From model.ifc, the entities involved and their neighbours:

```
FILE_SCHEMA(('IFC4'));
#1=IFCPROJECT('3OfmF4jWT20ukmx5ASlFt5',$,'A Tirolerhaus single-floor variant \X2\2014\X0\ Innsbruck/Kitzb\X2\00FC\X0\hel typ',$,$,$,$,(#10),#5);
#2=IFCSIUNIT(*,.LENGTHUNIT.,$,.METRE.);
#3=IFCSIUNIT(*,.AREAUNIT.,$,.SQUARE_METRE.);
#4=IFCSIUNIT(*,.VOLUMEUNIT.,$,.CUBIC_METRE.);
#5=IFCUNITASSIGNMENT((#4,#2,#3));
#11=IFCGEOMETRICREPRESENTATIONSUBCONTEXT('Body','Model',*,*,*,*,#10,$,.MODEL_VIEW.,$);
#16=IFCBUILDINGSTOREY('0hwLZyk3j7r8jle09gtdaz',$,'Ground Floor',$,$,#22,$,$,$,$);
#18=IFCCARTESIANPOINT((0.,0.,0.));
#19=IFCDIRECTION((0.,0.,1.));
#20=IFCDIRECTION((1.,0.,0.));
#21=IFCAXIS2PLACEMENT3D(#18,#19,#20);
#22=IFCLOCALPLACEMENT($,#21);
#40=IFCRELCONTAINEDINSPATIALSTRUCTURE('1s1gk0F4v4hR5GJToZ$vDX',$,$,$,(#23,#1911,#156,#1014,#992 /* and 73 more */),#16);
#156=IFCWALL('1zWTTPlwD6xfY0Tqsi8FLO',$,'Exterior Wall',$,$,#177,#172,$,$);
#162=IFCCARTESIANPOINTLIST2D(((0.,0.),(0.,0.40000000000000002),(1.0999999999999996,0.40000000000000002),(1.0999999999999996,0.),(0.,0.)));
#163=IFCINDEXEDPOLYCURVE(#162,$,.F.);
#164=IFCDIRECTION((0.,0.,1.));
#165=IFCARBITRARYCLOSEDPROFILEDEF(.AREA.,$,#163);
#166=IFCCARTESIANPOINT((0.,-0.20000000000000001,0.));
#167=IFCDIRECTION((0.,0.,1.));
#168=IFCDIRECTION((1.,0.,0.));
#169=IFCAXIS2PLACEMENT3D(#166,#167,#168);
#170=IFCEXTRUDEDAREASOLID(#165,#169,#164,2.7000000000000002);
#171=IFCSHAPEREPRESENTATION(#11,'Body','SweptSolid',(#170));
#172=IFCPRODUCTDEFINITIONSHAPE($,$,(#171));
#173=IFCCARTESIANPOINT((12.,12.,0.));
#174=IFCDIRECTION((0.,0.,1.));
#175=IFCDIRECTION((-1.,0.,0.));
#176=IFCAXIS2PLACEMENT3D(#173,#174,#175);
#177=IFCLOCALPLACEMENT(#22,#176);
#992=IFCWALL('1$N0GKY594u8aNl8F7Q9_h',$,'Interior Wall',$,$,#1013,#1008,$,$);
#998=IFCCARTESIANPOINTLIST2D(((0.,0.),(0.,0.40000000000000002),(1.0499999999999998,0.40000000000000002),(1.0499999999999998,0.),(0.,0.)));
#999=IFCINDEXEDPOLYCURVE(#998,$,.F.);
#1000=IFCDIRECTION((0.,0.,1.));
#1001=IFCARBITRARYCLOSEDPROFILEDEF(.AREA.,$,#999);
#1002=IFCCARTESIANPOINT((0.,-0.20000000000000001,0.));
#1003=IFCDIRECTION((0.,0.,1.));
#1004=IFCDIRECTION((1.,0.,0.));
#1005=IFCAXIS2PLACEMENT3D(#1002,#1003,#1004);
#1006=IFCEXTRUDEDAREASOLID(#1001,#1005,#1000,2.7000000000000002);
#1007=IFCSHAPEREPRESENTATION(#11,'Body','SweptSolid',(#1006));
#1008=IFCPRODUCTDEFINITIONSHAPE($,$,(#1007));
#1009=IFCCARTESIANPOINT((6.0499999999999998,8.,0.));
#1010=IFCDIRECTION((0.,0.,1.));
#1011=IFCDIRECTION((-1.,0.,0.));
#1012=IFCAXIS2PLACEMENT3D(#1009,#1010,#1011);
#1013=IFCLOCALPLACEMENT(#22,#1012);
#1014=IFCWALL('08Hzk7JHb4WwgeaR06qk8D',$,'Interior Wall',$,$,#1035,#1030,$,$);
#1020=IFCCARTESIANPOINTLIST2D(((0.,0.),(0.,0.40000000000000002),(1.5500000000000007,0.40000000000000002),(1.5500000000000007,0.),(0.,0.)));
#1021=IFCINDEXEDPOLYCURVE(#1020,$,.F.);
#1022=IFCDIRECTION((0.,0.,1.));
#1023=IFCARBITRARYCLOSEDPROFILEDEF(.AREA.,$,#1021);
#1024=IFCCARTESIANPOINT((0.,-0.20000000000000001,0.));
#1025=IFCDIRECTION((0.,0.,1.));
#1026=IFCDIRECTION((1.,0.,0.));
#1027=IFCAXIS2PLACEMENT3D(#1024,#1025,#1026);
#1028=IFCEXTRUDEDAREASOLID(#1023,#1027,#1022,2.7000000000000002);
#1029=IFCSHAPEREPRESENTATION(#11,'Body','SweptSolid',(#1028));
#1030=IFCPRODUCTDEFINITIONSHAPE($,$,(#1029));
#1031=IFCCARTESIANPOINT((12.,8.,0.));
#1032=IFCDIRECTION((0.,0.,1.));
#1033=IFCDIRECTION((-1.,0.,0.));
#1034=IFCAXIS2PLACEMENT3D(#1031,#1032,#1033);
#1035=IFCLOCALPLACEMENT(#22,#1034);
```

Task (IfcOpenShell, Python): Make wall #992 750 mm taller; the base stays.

```python
import ifcopenshell
import ifcopenshell.geom
import ifcopenshell.util.representation
import ifcopenshell.util.shape
import ifcopenshell.util.unit

model = ifcopenshell.open("model.ifc")
unit_scale = ifcopenshell.util.unit.calculate_unit_scale(model)
settings = ifcopenshell.geom.settings()


def volume(element):
    """Net volume in cubic metres, openings subtracted."""
    shape = ifcopenshell.geom.create_shape(settings, element)
    return ifcopenshell.util.shape.get_volume(shape.geometry)


wall = model.by_guid("1$N0GKY594u8aNl8F7Q9_h")
before = volume(wall)

body = ifcopenshell.util.representation.get_representation(wall, "Model", "Body")
solid = body.Items[0]
old_height = solid.Depth
solid.Depth += 0.75 / unit_scale
after = volume(wall)

print(f"height {old_height:g} -> {solid.Depth:g}, volume {before:.3f} -> {after:.3f} m3")

model.write("model_v2.ifc")
```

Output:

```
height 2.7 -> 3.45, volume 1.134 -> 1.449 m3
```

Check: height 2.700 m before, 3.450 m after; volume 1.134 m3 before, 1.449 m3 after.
